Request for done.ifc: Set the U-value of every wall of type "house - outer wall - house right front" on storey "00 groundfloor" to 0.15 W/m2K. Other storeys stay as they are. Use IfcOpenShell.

First a look at what the model holds.

```python
import ifcopenshell
import ifcopenshell.util.element

model = ifcopenshell.open("done.ifc")
print(model.schema)
storey = next(s for s in model.by_type("IfcBuildingStorey") if s.Name == "00 groundfloor")
walls = [e for e in ifcopenshell.util.element.get_decomposition(storey) if e.is_a("IfcWall")]
seen = {}
for e in walls:
    element_type = ifcopenshell.util.element.get_type(e)
    key = (element_type.Name if element_type != e and element_type else None, ifcopenshell.util.element.get_pset(e, "Pset_WallCommon", "ThermalTransmittance"))
    seen[key] = seen.get(key, 0) + 1
for (name, value), count in sorted(seen.items(), key=str):
    print(count, "x", name, "|", value)
```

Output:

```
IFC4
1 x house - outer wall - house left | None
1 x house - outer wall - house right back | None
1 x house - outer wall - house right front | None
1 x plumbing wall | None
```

```python
import ifcopenshell
import ifcopenshell.api.pset
import ifcopenshell.util.element

model = ifcopenshell.open("done.ifc")

storey = next(s for s in model.by_type("IfcBuildingStorey") if s.Name == "00 groundfloor")
walls = [e for e in ifcopenshell.util.element.get_decomposition(storey) if e.is_a("IfcWall")]

count = 0
for e in walls:
    element_type = ifcopenshell.util.element.get_type(e)
    if element_type in (None, e) or element_type.Name != "house - outer wall - house right front":
        continue
    # add_pset returns the element's existing set when there is one.
    pset = ifcopenshell.api.pset.add_pset(model, product=e, name="Pset_WallCommon")
    ifcopenshell.api.pset.edit_pset(model, pset=pset, properties={"ThermalTransmittance": 0.15})
    count += 1

print(count, "walls updated")

model.write("done_v2.ifc")
```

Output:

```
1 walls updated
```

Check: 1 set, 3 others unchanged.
